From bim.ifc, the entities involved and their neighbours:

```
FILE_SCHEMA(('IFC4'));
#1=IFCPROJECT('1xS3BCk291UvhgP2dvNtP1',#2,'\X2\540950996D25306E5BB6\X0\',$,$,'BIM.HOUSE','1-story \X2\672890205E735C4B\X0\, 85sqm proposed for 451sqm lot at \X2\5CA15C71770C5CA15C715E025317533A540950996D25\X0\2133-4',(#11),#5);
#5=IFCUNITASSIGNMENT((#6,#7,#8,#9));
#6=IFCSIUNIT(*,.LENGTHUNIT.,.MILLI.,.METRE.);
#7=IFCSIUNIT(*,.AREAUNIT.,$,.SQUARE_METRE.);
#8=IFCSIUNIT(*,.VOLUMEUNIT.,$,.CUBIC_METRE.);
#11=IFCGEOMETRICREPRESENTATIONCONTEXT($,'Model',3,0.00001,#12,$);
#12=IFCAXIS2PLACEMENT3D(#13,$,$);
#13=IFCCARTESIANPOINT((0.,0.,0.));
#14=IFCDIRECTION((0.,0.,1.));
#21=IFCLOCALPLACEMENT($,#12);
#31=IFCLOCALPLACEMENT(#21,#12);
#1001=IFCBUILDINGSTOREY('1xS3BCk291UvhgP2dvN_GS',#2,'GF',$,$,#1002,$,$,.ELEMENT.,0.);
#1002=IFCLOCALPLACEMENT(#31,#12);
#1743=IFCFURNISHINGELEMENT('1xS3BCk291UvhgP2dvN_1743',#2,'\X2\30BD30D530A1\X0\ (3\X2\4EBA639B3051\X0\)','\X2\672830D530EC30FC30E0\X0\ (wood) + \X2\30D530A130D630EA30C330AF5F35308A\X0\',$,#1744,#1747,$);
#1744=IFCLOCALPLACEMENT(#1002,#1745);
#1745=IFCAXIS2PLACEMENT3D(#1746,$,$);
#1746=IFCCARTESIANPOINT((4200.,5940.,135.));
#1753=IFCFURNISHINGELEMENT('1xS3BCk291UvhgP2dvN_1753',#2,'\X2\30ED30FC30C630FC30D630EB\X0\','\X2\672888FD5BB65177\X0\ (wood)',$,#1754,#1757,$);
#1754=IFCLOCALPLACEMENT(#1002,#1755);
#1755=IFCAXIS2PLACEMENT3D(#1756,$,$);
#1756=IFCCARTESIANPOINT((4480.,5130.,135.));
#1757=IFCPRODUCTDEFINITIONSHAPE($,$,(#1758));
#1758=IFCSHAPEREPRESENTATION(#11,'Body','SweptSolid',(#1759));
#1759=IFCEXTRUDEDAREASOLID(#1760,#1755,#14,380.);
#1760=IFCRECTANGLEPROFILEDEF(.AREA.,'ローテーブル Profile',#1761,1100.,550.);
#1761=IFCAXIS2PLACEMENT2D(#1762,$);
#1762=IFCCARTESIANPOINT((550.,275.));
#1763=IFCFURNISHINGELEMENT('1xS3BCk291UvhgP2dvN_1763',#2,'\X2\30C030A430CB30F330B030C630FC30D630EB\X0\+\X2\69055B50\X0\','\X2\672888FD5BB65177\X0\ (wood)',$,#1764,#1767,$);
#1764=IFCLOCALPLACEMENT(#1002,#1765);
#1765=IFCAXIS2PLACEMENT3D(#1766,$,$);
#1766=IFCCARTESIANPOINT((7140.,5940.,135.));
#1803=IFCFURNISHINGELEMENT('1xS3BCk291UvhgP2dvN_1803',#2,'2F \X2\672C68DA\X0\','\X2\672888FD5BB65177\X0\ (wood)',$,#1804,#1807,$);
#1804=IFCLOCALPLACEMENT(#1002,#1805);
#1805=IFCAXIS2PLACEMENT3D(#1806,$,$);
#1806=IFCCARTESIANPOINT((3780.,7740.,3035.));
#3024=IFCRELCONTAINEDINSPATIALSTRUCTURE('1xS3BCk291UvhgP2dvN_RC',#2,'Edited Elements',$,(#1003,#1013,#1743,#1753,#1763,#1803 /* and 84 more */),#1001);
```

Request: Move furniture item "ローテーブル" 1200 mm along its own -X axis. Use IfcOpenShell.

```python
import ifcopenshell
import ifcopenshell.api.geometry
import ifcopenshell.util.placement
import ifcopenshell.util.unit

model = ifcopenshell.open("bim.ifc")
unit_scale = ifcopenshell.util.unit.calculate_unit_scale(model)

item = model.by_id(1753)
matrix = ifcopenshell.util.placement.get_local_placement(item.ObjectPlacement)
matrix[:3, 3] -= matrix[:3, 0] * 1.2 / unit_scale
ifcopenshell.api.geometry.edit_object_placement(model, product=item, matrix=matrix, is_si=False)

print(ifcopenshell.util.placement.get_local_placement(item.ObjectPlacement).round(3) + 0.0)

model.write("bim_rev.ifc")
```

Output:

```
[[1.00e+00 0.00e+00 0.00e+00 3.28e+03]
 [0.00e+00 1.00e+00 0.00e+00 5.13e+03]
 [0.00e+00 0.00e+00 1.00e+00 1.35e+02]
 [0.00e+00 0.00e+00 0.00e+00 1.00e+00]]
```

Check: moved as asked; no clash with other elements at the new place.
